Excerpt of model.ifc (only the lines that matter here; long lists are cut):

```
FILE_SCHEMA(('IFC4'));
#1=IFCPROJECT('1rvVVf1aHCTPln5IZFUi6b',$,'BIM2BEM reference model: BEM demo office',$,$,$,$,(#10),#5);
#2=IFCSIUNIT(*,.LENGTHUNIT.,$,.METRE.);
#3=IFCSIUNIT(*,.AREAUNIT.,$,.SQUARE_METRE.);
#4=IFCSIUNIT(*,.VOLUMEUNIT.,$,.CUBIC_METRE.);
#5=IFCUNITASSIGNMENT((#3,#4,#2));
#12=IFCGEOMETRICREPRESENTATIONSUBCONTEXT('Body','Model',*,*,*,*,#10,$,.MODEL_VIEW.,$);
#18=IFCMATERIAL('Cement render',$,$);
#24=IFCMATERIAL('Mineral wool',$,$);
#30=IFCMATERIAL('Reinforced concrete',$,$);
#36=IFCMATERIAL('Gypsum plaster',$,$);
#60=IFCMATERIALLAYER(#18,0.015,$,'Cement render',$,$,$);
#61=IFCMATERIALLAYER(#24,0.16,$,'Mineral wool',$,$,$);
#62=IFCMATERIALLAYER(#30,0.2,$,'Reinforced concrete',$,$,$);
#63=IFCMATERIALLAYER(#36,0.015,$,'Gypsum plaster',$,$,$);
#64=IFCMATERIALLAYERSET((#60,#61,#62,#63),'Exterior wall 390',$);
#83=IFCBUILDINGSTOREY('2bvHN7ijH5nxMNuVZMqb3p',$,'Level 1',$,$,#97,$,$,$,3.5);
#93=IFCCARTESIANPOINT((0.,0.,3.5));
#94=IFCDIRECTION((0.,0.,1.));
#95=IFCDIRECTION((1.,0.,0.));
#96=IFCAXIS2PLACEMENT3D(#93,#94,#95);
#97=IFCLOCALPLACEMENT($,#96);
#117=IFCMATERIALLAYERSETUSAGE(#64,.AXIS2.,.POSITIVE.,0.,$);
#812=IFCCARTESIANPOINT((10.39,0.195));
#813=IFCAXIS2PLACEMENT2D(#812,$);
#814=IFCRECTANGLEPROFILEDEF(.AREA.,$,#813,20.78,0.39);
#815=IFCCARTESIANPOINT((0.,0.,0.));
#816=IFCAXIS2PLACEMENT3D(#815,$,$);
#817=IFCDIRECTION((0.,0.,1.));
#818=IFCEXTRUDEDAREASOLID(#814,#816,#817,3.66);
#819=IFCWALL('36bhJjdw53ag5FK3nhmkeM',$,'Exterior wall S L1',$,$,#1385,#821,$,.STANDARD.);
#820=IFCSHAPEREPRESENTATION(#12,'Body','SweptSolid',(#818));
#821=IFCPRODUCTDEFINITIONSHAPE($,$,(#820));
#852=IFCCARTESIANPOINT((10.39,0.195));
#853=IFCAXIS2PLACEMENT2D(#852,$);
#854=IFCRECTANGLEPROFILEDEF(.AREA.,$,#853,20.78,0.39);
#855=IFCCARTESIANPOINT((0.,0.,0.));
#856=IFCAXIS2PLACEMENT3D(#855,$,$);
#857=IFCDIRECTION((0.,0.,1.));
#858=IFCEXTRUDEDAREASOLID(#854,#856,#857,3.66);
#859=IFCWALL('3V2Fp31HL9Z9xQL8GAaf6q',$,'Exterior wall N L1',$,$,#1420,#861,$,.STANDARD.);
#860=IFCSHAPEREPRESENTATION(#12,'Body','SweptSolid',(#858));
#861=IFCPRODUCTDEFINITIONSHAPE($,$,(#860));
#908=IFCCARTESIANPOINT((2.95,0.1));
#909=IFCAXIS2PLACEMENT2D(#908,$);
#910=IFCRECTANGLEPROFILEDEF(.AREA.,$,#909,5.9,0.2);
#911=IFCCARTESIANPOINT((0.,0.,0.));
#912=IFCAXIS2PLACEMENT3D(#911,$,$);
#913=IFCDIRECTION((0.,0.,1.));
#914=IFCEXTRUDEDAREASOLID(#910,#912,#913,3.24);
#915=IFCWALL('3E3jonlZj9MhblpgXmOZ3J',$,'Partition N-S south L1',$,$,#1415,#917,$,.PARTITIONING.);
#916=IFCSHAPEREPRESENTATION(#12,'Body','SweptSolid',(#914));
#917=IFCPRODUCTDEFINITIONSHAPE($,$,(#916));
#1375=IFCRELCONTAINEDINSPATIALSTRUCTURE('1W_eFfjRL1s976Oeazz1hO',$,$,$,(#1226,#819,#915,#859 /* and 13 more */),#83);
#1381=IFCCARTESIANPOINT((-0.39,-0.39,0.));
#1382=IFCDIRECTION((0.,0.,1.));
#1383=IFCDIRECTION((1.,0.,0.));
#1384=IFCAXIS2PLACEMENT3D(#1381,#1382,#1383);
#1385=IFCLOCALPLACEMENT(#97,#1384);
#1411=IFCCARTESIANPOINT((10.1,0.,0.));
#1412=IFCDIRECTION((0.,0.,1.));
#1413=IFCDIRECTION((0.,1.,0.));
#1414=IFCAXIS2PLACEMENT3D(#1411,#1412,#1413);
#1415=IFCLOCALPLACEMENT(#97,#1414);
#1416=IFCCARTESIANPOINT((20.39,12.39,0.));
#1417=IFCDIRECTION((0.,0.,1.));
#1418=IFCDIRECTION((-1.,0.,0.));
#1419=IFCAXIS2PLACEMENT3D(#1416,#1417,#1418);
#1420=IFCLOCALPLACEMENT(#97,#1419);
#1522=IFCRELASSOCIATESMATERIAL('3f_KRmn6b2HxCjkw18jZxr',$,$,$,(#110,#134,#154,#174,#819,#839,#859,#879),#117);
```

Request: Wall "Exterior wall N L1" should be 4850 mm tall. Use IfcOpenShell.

```python
import ifcopenshell
import ifcopenshell.geom
import ifcopenshell.util.representation
import ifcopenshell.util.shape
import ifcopenshell.util.unit

model = ifcopenshell.open("model.ifc")
unit_scale = ifcopenshell.util.unit.calculate_unit_scale(model)
settings = ifcopenshell.geom.settings()


def volume(element):
    """Net volume in cubic metres, openings subtracted."""
    shape = ifcopenshell.geom.create_shape(settings, element)
    return ifcopenshell.util.shape.get_volume(shape.geometry)


wall = model.by_id(859)
before = volume(wall)

body = ifcopenshell.util.representation.get_representation(wall, "Model", "Body")
solid = body.Items[0]
old_height = solid.Depth
solid.Depth = 4.85 / unit_scale
after = volume(wall)

print(f"height {old_height:g} -> {solid.Depth:g}, volume {before:.3f} -> {after:.3f} m3")

model.write("model_rev.ifc")
```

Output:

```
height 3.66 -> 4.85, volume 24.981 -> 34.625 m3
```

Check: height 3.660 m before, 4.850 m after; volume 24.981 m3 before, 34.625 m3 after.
